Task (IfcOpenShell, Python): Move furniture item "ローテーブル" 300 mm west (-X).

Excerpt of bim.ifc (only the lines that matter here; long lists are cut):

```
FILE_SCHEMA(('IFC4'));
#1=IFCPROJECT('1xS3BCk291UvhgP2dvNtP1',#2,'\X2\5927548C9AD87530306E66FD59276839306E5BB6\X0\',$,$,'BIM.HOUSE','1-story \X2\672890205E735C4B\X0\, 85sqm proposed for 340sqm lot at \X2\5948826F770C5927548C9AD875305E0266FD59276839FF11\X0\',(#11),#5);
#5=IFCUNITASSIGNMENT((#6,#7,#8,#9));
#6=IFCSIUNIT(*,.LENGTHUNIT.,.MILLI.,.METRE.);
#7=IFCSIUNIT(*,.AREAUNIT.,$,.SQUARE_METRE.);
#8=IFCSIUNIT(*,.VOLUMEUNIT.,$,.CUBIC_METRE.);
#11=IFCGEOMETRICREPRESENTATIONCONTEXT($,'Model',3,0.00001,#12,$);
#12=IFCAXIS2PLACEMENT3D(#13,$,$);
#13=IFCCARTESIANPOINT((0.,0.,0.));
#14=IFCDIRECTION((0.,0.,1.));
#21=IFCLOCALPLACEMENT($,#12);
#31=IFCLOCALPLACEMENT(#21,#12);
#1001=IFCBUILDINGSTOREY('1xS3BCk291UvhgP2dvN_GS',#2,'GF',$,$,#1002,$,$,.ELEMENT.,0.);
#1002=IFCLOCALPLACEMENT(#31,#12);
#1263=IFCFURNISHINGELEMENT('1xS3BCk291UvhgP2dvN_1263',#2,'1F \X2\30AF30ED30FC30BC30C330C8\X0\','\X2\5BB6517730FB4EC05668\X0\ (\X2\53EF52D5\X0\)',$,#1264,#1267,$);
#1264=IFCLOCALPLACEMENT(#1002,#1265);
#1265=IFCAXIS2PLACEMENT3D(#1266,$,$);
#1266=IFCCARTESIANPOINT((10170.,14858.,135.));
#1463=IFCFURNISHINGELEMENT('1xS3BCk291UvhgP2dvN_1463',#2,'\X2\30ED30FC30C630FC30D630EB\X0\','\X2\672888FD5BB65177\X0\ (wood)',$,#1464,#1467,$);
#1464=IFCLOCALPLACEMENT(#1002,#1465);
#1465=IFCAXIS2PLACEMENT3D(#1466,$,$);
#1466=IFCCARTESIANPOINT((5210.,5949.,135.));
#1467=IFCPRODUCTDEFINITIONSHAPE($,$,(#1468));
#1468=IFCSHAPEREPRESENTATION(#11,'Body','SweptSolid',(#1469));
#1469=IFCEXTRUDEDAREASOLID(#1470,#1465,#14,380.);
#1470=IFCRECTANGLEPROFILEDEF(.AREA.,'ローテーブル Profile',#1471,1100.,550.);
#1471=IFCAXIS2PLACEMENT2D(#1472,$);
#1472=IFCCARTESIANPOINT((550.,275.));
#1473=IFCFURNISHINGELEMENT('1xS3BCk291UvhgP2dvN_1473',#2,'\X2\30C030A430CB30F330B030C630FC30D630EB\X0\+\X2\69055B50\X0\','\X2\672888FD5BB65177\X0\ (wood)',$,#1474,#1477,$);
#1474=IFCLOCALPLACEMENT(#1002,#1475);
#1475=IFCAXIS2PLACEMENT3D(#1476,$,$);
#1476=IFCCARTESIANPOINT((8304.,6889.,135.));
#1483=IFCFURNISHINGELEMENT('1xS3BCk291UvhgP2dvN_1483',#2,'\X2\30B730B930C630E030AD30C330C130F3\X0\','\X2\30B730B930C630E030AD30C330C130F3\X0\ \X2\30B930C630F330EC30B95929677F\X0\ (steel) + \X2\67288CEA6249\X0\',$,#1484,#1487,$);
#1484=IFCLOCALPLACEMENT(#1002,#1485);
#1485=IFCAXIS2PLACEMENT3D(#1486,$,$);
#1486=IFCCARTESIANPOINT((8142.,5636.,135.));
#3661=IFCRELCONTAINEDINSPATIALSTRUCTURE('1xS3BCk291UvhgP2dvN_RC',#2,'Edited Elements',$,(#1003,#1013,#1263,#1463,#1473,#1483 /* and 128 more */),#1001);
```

```python
import ifcopenshell
import ifcopenshell.api.geometry
import ifcopenshell.util.placement
import ifcopenshell.util.unit

model = ifcopenshell.open("bim.ifc")
unit_scale = ifcopenshell.util.unit.calculate_unit_scale(model)

item = model.by_id(1463)
matrix = ifcopenshell.util.placement.get_local_placement(item.ObjectPlacement)
matrix[0, 3] -= 0.3 / unit_scale
ifcopenshell.api.geometry.edit_object_placement(model, product=item, matrix=matrix, is_si=False)

print(ifcopenshell.util.placement.get_local_placement(item.ObjectPlacement).round(3) + 0.0)

model.write("bim_rev.ifc")
```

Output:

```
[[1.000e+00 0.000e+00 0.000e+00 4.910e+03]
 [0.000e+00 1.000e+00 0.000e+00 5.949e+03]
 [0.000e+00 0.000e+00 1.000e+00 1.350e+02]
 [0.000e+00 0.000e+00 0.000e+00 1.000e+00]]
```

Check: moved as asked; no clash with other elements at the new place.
